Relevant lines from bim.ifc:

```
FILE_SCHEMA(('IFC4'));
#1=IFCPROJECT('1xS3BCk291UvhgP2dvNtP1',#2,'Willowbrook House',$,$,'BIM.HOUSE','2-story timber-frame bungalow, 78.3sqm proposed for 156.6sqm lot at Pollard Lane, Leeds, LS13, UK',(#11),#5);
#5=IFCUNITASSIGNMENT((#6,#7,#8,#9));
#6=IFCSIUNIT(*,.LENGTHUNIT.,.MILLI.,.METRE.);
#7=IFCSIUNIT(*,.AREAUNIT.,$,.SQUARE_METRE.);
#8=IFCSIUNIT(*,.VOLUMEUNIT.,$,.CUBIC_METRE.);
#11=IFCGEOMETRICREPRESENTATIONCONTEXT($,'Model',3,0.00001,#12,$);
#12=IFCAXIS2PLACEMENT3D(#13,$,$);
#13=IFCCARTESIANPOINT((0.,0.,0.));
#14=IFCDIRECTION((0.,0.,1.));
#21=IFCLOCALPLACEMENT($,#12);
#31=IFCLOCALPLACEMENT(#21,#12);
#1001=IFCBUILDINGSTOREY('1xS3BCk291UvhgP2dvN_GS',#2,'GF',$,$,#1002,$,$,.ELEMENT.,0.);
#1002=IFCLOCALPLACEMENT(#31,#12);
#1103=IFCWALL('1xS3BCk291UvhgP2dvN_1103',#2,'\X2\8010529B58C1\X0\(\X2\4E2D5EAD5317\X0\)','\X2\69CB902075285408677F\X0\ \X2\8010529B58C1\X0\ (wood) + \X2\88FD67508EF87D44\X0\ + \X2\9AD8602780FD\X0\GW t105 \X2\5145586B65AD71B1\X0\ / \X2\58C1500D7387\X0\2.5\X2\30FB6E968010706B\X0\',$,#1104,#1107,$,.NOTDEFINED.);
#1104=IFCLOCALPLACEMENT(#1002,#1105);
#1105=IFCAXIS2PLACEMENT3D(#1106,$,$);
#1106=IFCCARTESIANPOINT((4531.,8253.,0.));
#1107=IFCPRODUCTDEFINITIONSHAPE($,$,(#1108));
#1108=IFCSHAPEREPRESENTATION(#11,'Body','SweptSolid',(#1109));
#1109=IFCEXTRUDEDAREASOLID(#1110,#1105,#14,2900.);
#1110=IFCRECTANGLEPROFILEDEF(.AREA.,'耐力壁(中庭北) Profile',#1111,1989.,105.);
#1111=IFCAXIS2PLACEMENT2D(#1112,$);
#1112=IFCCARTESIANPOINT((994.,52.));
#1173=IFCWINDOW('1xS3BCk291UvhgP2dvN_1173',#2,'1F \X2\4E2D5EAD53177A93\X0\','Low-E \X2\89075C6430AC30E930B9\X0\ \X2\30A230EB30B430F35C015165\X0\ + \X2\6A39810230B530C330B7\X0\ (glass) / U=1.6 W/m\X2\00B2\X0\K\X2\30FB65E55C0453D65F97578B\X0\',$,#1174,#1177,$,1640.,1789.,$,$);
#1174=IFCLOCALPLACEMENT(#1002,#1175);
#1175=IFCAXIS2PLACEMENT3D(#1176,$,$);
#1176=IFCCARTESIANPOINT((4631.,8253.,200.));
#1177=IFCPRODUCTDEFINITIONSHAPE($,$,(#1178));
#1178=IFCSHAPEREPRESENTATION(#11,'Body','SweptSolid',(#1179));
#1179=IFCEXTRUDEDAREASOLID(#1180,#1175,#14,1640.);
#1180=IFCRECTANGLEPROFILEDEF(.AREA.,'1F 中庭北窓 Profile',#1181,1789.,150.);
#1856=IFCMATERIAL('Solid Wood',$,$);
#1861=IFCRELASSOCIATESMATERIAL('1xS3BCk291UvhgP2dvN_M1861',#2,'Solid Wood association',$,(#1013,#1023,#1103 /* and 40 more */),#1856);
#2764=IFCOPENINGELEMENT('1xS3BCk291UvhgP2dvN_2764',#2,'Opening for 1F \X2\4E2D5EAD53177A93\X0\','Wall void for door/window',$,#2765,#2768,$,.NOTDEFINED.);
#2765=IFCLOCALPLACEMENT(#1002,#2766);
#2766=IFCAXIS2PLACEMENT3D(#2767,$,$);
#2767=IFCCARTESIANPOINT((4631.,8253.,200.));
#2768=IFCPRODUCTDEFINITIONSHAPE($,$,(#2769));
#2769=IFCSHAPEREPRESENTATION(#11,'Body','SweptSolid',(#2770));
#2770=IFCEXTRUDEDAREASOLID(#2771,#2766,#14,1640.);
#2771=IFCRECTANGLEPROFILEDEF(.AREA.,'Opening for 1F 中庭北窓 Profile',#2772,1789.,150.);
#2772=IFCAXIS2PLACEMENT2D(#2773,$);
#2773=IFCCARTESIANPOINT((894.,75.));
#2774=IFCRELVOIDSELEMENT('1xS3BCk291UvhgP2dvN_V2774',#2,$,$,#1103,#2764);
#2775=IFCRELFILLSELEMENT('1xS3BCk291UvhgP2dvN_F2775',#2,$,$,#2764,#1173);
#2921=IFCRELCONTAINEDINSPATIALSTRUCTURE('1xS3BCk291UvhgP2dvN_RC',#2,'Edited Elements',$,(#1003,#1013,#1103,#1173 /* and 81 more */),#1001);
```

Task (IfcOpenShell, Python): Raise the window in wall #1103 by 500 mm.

```python
import numpy as np
import ifcopenshell
import ifcopenshell.api.geometry
import ifcopenshell.util.placement
import ifcopenshell.util.unit

model = ifcopenshell.open("bim.ifc")
unit_scale = ifcopenshell.util.unit.calculate_unit_scale(model)

window = model.by_guid("1xS3BCk291UvhgP2dvN_1173")
opening = window.FillsVoids[0].RelatingOpeningElement
dz = 0.5 / unit_scale

shift = np.array([0.0, 0.0, dz])
# The window is not placed relative to its opening, so move both.
for product in (opening, window):
    matrix = ifcopenshell.util.placement.get_local_placement(product.ObjectPlacement)
    matrix[:3, 3] += shift
    ifcopenshell.api.geometry.edit_object_placement(model, product=product, matrix=matrix, is_si=False)

print(f"moved by {dz * unit_scale:+.3f} m")

model.write("bim_edited.ifc")
```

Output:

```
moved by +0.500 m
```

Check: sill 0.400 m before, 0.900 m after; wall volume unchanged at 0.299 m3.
